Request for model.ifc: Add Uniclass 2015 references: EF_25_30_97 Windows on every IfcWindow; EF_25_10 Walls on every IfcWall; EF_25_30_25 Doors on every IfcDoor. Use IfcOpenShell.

First a look at what the model holds.

```python
import ifcopenshell

model = ifcopenshell.open("model.ifc")
print(model.schema)
print("classifications:", [c.Name for c in model.by_type("IfcClassification")])
for ifc_class in ("IfcDoor", "IfcRoof", "IfcStair", "IfcWall", "IfcWindow"):
    print(ifc_class, len(model.by_type(ifc_class)))
```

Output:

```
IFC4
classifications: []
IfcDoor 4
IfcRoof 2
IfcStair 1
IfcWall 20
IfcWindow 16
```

```python
import ifcopenshell
import ifcopenshell.api.classification

model = ifcopenshell.open("model.ifc")

system = ifcopenshell.api.classification.add_classification(model, classification="Uniclass 2015")

codes = {
    "IfcWindow": ("EF_25_30_97", "Windows"),
    "IfcWall": ("EF_25_10", "Walls"),
    "IfcDoor": ("EF_25_30_25", "Doors"),
}
for ifc_class, (code, name) in codes.items():
    products = model.by_type(ifc_class)
    ifcopenshell.api.classification.add_reference(
        model, products=products, classification=system, identification=code, name=name
    )
    print(code, len(products))

model.write("model_v2.ifc")
```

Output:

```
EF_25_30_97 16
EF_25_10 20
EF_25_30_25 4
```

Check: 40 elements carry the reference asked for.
